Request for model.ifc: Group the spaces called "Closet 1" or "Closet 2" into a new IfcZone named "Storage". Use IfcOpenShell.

First a look at what the model holds.

```python
import ifcopenshell

model = ifcopenshell.open("model.ifc")
print(model.schema)
seen = {}
for space in model.by_type("IfcSpace"):
    seen[space.LongName] = seen.get(space.LongName, 0) + 1
for name, count in sorted(seen.items(), key=str):
    print(count, "x", name)
print("zones:", [z.Name for z in model.by_type("IfcZone")][:20])
```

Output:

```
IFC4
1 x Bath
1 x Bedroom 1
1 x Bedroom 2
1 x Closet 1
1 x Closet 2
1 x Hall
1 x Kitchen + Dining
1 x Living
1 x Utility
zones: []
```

```python
import ifcopenshell
import ifcopenshell.api.group
import ifcopenshell.api.root

model = ifcopenshell.open("model.ifc")

names = {"Closet 1", "Closet 2"}
spaces = [s for s in model.by_type("IfcSpace") if s.LongName in names]

zone = ifcopenshell.api.root.create_entity(model, ifc_class="IfcZone", name="Storage")
ifcopenshell.api.group.assign_group(model, products=spaces, group=zone)
print(len(spaces), "spaces in", zone.Name)

model.write("model_rev.ifc")
```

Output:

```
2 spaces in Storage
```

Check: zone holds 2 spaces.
